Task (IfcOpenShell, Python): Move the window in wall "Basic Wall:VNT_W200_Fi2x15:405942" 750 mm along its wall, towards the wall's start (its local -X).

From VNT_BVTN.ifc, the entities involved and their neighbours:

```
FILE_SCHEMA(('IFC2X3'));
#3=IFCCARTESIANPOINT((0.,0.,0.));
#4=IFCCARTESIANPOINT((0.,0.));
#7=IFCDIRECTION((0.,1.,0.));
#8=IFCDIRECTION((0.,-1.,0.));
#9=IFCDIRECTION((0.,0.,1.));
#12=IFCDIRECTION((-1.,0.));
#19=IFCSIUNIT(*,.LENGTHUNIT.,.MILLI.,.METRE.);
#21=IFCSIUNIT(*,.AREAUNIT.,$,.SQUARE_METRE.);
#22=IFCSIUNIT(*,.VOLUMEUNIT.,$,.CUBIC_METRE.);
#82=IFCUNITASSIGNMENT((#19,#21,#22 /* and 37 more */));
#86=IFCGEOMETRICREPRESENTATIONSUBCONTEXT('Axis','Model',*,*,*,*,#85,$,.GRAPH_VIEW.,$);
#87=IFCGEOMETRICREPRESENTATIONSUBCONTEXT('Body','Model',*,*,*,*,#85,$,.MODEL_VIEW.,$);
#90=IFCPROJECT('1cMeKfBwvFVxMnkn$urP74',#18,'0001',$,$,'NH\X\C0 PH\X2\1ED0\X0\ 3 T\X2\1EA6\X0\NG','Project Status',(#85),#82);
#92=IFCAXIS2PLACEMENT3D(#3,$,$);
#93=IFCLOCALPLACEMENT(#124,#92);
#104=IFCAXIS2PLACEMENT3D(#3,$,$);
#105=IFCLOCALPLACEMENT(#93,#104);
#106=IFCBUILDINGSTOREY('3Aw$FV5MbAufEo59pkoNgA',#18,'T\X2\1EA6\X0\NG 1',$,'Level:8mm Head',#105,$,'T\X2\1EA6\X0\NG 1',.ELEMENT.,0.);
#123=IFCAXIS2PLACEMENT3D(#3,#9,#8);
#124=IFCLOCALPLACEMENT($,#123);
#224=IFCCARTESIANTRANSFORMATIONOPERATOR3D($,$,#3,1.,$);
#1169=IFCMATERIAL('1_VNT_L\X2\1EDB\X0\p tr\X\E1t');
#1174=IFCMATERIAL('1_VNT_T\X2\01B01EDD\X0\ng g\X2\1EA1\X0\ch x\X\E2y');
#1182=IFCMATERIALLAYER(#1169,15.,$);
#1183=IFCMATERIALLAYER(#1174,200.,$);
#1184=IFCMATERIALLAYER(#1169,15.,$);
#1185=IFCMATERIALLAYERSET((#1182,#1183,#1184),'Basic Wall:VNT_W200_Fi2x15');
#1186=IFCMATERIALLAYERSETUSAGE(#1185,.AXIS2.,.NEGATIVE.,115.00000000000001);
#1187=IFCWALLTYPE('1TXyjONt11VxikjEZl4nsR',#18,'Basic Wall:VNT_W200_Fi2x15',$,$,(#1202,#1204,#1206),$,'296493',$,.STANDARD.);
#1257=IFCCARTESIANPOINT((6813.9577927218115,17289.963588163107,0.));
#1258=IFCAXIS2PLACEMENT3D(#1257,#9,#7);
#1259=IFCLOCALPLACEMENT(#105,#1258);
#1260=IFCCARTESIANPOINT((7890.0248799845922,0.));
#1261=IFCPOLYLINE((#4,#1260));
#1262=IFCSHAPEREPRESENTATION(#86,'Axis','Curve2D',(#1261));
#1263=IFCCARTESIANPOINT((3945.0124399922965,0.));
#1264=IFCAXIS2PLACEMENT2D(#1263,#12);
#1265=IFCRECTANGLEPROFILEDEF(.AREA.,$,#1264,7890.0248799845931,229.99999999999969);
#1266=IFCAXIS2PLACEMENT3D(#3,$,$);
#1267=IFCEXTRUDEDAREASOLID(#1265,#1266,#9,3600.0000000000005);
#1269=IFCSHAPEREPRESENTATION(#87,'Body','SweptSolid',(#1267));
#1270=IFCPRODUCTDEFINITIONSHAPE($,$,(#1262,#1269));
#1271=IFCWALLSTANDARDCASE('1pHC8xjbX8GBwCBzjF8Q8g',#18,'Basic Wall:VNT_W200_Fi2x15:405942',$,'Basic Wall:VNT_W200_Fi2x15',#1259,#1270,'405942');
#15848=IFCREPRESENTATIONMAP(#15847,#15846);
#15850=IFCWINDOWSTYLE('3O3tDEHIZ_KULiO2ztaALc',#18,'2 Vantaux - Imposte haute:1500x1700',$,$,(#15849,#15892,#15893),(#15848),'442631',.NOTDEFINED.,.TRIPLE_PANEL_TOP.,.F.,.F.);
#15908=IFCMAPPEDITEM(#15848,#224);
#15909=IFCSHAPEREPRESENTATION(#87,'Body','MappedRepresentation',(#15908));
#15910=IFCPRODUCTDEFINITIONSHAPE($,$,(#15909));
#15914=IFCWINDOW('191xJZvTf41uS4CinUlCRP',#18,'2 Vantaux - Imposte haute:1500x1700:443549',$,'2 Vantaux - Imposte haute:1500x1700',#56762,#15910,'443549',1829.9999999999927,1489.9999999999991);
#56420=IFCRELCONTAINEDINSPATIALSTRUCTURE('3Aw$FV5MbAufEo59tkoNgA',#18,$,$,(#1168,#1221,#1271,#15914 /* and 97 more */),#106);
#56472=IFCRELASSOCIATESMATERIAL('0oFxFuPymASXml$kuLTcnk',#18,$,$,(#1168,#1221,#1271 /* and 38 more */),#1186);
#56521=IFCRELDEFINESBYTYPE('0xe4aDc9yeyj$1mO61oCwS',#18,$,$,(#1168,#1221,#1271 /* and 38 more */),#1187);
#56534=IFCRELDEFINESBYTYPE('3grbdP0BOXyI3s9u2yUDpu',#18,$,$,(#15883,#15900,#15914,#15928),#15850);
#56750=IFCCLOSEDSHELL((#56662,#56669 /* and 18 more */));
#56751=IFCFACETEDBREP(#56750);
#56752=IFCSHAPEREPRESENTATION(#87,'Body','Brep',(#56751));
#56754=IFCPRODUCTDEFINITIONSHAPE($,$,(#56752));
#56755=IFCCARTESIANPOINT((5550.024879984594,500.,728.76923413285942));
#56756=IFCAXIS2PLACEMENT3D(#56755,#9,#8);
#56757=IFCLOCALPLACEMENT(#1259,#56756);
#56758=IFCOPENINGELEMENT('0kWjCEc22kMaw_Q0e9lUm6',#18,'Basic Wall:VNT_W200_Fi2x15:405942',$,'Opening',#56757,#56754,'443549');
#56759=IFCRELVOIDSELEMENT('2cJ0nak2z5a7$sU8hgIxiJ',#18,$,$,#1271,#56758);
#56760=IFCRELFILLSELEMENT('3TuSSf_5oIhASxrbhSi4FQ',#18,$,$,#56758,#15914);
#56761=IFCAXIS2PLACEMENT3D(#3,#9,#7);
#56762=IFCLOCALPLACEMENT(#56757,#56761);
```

```python
import ifcopenshell
import ifcopenshell.api.geometry
import ifcopenshell.util.placement
import ifcopenshell.util.unit

model = ifcopenshell.open("VNT_BVTN.ifc")
unit_scale = ifcopenshell.util.unit.calculate_unit_scale(model)

window = model.by_guid("191xJZvTf41uS4CinUlCRP")
opening = window.FillsVoids[0].RelatingOpeningElement
wall = opening.VoidsElements[0].RelatingBuildingElement

wall_matrix = ifcopenshell.util.placement.get_local_placement(wall.ObjectPlacement)
shift = wall_matrix[:3, 0] * -0.75 / unit_scale
before = ifcopenshell.util.placement.get_local_placement(window.ObjectPlacement)[:3, 3].copy()

# The window is placed relative to its opening, so it follows when the opening moves.
matrix = ifcopenshell.util.placement.get_local_placement(opening.ObjectPlacement)
matrix[:3, 3] += shift
ifcopenshell.api.geometry.edit_object_placement(
    model, product=opening, matrix=matrix, is_si=False, should_transform_children=True
)

after = ifcopenshell.util.placement.get_local_placement(window.ObjectPlacement)[:3, 3]
print("window moved by", (after - before).round(3) + 0.0)

model.write("VNT_BVTN-out.ifc")
```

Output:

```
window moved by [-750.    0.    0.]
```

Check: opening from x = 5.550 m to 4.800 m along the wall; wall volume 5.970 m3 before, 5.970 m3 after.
